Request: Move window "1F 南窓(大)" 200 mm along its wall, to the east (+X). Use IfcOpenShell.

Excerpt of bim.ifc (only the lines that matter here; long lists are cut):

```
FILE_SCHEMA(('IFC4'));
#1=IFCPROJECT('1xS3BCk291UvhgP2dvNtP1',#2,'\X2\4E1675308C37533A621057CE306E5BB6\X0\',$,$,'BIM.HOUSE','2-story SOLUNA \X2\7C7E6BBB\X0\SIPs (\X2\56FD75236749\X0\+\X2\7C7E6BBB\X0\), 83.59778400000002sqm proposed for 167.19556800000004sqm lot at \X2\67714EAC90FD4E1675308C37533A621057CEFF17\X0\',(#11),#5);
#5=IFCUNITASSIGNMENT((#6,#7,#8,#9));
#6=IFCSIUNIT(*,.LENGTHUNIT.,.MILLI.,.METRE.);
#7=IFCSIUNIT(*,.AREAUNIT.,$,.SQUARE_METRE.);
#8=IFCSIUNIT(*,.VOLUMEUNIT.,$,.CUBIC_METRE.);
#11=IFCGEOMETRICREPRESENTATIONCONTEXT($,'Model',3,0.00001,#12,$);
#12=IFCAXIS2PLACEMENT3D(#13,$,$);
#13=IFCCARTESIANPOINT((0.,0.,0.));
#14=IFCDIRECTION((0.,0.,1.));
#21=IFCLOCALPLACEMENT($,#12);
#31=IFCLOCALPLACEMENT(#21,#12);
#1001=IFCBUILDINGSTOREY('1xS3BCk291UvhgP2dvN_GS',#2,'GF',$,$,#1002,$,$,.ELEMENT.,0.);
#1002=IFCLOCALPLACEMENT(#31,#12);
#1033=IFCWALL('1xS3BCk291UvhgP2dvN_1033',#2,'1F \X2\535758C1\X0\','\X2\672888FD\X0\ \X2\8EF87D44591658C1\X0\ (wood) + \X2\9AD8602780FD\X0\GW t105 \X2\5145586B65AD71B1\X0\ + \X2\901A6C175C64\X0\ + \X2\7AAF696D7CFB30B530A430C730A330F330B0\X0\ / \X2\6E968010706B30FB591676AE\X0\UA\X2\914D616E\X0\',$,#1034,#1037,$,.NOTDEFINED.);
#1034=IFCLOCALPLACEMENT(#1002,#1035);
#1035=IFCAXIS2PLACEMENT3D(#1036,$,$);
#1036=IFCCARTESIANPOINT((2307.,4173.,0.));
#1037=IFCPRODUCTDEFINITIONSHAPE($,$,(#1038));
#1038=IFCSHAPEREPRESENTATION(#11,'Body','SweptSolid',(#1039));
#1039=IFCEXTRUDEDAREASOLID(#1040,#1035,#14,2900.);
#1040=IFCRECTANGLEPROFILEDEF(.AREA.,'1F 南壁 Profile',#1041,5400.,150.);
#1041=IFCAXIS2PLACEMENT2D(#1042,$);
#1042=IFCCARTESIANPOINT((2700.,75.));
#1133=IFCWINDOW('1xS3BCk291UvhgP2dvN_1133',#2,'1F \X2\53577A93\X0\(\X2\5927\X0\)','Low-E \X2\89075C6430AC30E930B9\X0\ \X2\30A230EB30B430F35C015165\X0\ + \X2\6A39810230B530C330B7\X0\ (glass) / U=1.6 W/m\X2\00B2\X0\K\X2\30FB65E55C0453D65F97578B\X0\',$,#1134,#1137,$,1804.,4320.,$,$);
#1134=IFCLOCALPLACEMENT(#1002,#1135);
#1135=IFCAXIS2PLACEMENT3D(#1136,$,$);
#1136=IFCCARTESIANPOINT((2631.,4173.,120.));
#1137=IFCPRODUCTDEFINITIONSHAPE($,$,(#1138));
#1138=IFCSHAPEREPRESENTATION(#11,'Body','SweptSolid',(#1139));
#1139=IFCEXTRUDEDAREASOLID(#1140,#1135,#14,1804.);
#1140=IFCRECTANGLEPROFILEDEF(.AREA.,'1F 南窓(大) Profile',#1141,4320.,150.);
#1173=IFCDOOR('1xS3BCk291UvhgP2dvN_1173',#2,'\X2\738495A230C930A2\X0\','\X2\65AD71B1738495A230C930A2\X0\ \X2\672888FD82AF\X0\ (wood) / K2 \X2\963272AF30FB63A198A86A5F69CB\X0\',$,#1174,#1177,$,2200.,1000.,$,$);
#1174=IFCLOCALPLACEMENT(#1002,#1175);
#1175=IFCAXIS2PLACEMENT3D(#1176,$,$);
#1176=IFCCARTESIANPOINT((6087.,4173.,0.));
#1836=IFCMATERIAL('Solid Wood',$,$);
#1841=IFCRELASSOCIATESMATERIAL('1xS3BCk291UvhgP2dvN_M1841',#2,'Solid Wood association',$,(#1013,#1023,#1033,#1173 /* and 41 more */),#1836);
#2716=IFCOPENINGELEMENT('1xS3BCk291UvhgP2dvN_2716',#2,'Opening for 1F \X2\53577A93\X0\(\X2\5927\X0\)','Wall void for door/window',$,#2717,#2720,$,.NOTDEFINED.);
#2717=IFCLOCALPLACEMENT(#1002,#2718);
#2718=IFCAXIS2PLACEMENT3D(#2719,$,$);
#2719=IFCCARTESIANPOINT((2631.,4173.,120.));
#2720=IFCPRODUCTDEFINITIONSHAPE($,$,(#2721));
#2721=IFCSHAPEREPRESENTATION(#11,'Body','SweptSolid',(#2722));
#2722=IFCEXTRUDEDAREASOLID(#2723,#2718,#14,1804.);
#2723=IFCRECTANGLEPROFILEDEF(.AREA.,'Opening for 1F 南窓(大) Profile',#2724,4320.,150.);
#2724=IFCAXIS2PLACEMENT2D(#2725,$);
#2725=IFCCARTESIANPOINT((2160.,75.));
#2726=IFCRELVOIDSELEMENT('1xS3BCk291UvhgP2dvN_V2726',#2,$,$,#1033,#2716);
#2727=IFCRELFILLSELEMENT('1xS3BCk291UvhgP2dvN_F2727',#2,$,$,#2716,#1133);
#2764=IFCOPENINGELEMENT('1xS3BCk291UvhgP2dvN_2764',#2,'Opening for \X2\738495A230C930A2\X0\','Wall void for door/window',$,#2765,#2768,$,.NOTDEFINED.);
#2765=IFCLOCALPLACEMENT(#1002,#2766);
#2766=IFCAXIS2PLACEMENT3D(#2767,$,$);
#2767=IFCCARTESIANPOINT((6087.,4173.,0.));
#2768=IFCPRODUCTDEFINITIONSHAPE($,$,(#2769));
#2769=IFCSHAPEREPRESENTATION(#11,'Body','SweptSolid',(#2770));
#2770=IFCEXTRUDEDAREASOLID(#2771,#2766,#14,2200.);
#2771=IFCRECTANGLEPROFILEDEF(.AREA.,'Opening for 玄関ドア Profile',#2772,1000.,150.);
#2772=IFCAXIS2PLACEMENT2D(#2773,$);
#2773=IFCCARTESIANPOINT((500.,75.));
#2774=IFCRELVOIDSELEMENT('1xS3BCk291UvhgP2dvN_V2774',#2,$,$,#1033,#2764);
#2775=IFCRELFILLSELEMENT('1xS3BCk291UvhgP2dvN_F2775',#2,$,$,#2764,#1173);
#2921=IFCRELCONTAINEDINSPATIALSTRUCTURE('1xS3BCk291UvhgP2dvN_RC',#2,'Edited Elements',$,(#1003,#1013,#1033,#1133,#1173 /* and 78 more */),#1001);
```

```python
import ifcopenshell
import ifcopenshell.api.geometry
import ifcopenshell.util.placement

model = ifcopenshell.open("bim.ifc")

window = model.by_id(1133)
opening = window.FillsVoids[0].RelatingOpeningElement
wall = opening.VoidsElements[0].RelatingBuildingElement

wall_matrix = ifcopenshell.util.placement.get_local_placement(wall.ObjectPlacement)
shift = wall_matrix[:3, 0] * 200.0
before = ifcopenshell.util.placement.get_local_placement(window.ObjectPlacement)[:3, 3].copy()

# The window is not placed relative to its opening, so move both.
for product in (opening, window):
    matrix = ifcopenshell.util.placement.get_local_placement(product.ObjectPlacement)
    matrix[:3, 3] += shift
    ifcopenshell.api.geometry.edit_object_placement(model, product=product, matrix=matrix, is_si=False)

after = ifcopenshell.util.placement.get_local_placement(window.ObjectPlacement)[:3, 3]
print("window moved by", (after - before).round(3) + 0.0)

model.write("bim_rev.ifc")
```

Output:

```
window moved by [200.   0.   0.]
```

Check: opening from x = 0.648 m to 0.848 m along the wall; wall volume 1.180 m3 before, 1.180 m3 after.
